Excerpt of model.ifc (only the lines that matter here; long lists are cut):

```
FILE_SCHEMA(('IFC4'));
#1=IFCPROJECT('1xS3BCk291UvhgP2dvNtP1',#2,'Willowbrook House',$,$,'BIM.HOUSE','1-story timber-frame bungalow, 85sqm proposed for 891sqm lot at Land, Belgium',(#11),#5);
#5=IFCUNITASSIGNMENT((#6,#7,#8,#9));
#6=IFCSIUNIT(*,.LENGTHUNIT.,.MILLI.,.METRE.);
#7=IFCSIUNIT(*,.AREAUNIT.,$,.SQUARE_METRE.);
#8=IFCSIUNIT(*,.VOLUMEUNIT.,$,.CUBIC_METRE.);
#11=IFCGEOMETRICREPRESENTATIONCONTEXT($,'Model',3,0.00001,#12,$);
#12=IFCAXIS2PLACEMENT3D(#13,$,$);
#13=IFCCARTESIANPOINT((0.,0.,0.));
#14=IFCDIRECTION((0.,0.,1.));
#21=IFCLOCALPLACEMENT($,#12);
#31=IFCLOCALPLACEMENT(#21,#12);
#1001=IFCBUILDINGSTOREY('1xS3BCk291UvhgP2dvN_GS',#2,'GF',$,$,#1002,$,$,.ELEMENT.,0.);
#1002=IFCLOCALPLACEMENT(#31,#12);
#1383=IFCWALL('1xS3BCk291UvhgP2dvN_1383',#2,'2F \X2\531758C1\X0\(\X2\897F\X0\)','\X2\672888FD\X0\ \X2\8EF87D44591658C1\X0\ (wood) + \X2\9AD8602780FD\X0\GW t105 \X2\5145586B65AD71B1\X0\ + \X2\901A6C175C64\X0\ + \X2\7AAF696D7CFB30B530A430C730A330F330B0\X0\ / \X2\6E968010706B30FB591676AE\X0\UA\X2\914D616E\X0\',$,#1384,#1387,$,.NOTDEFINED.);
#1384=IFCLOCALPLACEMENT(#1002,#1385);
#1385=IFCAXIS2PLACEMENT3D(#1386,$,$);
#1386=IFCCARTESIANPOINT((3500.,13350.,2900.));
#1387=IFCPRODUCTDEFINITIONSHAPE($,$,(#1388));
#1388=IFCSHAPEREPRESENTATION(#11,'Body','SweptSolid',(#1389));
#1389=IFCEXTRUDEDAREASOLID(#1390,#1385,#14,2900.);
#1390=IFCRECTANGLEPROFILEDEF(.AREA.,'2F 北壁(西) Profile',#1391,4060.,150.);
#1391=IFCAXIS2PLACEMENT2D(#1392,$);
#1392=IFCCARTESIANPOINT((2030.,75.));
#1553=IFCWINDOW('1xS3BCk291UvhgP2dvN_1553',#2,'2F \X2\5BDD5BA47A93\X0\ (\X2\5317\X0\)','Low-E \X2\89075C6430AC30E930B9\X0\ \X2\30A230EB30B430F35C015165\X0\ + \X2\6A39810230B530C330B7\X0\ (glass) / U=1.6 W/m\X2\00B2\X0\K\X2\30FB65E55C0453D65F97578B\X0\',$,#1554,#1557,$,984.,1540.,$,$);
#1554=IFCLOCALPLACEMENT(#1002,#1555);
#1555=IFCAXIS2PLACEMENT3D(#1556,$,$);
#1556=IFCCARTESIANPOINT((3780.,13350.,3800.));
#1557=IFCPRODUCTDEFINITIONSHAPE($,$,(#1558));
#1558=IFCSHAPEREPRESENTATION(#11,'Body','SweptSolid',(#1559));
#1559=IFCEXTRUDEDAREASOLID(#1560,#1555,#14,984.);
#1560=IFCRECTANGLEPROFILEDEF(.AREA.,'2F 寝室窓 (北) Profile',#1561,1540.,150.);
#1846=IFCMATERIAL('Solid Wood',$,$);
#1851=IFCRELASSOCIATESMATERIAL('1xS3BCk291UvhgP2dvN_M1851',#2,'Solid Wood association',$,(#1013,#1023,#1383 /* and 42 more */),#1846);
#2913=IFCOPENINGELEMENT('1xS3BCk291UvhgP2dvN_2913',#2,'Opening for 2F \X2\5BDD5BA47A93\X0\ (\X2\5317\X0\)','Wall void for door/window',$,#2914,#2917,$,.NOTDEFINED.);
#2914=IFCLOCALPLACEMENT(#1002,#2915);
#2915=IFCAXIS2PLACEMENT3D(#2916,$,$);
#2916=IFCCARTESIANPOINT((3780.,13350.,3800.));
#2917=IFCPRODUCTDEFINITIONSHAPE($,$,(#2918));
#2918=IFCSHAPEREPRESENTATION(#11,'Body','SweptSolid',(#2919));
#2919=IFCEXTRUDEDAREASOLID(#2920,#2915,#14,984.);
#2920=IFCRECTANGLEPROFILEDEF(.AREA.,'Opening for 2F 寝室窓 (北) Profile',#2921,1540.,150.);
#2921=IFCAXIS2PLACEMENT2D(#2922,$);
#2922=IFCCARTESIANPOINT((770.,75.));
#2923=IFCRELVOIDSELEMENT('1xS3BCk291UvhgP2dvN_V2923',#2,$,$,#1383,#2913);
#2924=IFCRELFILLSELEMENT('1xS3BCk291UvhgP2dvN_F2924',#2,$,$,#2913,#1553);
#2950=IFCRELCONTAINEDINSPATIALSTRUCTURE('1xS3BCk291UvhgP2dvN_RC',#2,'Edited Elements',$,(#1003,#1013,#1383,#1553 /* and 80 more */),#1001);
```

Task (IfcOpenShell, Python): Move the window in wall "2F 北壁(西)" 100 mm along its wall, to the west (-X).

```python
import ifcopenshell
import ifcopenshell.api.geometry
import ifcopenshell.util.placement
import ifcopenshell.util.unit

model = ifcopenshell.open("model.ifc")
unit_scale = ifcopenshell.util.unit.calculate_unit_scale(model)

window = model.by_guid("1xS3BCk291UvhgP2dvN_1553")
opening = window.FillsVoids[0].RelatingOpeningElement
wall = opening.VoidsElements[0].RelatingBuildingElement

wall_matrix = ifcopenshell.util.placement.get_local_placement(wall.ObjectPlacement)
shift = wall_matrix[:3, 0] * -0.1 / unit_scale
before = ifcopenshell.util.placement.get_local_placement(window.ObjectPlacement)[:3, 3].copy()

# The window is not placed relative to its opening, so move both.
for product in (opening, window):
    matrix = ifcopenshell.util.placement.get_local_placement(product.ObjectPlacement)
    matrix[:3, 3] += shift
    ifcopenshell.api.geometry.edit_object_placement(model, product=product, matrix=matrix, is_si=False)

after = ifcopenshell.util.placement.get_local_placement(window.ObjectPlacement)[:3, 3]
print("window moved by", (after - before).round(3) + 0.0)

model.write("model_edited.ifc")
```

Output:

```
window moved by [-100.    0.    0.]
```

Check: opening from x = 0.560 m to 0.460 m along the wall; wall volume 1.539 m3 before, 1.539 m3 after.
